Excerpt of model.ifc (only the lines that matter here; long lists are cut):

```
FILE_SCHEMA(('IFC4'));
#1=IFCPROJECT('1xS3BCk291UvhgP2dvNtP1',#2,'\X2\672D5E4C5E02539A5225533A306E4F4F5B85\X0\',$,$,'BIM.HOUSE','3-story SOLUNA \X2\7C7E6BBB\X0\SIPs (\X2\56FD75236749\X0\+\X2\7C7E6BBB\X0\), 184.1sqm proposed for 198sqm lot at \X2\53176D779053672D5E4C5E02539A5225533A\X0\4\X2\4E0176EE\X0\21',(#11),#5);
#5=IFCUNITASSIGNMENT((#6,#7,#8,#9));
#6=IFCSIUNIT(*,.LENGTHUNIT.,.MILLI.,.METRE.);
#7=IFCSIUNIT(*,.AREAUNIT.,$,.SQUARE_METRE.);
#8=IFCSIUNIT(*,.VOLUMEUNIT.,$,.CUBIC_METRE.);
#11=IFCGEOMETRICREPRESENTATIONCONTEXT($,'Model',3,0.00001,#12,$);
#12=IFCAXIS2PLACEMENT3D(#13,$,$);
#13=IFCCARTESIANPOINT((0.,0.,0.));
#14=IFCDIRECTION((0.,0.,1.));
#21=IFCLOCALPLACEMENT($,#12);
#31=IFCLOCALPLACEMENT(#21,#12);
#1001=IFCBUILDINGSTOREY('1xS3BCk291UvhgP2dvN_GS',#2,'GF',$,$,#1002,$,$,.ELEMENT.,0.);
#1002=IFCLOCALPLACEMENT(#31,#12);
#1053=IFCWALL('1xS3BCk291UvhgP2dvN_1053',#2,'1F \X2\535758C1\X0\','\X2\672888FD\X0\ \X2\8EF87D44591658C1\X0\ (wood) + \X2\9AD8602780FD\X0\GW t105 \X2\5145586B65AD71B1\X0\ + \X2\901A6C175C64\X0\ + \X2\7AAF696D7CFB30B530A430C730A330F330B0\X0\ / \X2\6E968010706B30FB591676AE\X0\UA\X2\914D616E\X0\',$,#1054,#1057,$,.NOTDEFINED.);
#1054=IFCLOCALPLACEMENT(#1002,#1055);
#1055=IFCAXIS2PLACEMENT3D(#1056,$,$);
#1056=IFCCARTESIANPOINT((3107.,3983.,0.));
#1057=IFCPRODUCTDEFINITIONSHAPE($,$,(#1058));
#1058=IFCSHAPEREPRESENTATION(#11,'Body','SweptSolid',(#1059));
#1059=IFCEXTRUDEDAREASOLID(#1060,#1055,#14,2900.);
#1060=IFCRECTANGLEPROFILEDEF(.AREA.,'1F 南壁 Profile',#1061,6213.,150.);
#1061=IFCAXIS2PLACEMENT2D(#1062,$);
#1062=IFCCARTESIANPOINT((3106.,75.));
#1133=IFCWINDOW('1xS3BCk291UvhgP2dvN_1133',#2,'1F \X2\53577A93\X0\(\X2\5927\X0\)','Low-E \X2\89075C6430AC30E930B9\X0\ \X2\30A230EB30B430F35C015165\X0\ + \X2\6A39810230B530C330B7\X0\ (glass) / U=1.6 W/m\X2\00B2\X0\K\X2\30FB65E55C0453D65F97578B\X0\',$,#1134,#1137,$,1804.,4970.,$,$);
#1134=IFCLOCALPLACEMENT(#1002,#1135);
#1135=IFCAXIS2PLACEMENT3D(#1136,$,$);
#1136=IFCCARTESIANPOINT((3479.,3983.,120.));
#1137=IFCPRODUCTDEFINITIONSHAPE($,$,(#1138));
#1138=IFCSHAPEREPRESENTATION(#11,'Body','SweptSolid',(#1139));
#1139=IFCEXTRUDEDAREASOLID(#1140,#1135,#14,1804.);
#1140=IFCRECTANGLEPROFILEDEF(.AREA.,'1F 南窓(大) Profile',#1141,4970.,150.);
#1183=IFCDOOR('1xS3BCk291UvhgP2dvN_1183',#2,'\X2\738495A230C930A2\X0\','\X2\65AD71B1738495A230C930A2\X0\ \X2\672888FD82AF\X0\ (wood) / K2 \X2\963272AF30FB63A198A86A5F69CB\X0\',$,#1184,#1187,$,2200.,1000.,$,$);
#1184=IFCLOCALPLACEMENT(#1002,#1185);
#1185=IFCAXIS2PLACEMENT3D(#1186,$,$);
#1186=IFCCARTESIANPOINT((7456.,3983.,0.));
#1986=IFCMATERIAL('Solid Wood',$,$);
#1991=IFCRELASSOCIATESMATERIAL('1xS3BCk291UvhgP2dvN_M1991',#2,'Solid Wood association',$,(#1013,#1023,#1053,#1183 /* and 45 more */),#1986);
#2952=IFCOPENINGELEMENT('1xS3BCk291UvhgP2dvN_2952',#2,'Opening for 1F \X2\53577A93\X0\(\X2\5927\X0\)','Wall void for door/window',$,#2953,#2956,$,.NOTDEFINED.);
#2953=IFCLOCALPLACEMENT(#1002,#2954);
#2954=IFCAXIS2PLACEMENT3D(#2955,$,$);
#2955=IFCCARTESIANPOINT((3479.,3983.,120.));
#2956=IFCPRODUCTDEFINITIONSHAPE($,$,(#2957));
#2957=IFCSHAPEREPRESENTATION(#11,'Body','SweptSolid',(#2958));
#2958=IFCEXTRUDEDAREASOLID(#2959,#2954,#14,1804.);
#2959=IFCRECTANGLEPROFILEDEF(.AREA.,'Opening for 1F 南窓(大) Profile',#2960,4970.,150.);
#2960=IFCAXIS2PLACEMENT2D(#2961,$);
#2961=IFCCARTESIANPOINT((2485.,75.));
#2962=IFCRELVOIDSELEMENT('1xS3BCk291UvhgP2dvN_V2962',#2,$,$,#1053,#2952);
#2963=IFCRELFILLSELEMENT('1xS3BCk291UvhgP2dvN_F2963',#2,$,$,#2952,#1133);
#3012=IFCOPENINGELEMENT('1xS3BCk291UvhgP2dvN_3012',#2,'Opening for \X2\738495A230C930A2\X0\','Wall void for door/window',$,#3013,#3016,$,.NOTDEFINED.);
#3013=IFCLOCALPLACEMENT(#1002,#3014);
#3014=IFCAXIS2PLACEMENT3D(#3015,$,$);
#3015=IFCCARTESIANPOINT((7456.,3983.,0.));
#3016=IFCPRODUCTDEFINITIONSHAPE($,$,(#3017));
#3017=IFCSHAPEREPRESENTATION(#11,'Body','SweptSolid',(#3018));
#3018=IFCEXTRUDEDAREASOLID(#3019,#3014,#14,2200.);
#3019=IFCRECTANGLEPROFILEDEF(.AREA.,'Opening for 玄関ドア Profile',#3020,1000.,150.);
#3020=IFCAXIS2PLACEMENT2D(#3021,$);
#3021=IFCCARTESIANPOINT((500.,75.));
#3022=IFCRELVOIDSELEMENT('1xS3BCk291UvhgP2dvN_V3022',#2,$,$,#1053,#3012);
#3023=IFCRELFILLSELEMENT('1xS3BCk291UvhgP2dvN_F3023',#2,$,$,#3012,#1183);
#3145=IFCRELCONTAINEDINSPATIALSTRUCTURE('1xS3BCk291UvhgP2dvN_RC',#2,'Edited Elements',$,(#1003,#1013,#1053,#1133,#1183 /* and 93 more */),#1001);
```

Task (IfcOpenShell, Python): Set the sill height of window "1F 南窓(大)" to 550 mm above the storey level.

```python
import numpy as np
import ifcopenshell
import ifcopenshell.api.geometry
import ifcopenshell.geom
import ifcopenshell.util.element
import ifcopenshell.util.placement
import ifcopenshell.util.shape
import ifcopenshell.util.unit

model = ifcopenshell.open("model.ifc")
unit_scale = ifcopenshell.util.unit.calculate_unit_scale(model)

window = model.by_id(1133)
opening = window.FillsVoids[0].RelatingOpeningElement
storey = ifcopenshell.util.element.get_container(window, ifc_class="IfcBuildingStorey")
level = ifcopenshell.util.placement.get_local_placement(storey.ObjectPlacement)[2, 3]

# The opening's origin need not be at the sill, so measure its lowest point.
shape = ifcopenshell.geom.create_shape(ifcopenshell.geom.settings(), opening)
bottom = ifcopenshell.util.shape.get_shape_bottom_elevation(shape, shape.geometry) / unit_scale
dz = level + 0.55 / unit_scale - bottom

shift = np.array([0.0, 0.0, dz])
# The window is not placed relative to its opening, so move both.
for product in (opening, window):
    matrix = ifcopenshell.util.placement.get_local_placement(product.ObjectPlacement)
    matrix[:3, 3] += shift
    ifcopenshell.api.geometry.edit_object_placement(model, product=product, matrix=matrix, is_si=False)

print(f"moved by {dz * unit_scale:+.3f} m")

model.write("model-out.ifc")
```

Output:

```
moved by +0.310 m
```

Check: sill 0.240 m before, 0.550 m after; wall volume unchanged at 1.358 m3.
